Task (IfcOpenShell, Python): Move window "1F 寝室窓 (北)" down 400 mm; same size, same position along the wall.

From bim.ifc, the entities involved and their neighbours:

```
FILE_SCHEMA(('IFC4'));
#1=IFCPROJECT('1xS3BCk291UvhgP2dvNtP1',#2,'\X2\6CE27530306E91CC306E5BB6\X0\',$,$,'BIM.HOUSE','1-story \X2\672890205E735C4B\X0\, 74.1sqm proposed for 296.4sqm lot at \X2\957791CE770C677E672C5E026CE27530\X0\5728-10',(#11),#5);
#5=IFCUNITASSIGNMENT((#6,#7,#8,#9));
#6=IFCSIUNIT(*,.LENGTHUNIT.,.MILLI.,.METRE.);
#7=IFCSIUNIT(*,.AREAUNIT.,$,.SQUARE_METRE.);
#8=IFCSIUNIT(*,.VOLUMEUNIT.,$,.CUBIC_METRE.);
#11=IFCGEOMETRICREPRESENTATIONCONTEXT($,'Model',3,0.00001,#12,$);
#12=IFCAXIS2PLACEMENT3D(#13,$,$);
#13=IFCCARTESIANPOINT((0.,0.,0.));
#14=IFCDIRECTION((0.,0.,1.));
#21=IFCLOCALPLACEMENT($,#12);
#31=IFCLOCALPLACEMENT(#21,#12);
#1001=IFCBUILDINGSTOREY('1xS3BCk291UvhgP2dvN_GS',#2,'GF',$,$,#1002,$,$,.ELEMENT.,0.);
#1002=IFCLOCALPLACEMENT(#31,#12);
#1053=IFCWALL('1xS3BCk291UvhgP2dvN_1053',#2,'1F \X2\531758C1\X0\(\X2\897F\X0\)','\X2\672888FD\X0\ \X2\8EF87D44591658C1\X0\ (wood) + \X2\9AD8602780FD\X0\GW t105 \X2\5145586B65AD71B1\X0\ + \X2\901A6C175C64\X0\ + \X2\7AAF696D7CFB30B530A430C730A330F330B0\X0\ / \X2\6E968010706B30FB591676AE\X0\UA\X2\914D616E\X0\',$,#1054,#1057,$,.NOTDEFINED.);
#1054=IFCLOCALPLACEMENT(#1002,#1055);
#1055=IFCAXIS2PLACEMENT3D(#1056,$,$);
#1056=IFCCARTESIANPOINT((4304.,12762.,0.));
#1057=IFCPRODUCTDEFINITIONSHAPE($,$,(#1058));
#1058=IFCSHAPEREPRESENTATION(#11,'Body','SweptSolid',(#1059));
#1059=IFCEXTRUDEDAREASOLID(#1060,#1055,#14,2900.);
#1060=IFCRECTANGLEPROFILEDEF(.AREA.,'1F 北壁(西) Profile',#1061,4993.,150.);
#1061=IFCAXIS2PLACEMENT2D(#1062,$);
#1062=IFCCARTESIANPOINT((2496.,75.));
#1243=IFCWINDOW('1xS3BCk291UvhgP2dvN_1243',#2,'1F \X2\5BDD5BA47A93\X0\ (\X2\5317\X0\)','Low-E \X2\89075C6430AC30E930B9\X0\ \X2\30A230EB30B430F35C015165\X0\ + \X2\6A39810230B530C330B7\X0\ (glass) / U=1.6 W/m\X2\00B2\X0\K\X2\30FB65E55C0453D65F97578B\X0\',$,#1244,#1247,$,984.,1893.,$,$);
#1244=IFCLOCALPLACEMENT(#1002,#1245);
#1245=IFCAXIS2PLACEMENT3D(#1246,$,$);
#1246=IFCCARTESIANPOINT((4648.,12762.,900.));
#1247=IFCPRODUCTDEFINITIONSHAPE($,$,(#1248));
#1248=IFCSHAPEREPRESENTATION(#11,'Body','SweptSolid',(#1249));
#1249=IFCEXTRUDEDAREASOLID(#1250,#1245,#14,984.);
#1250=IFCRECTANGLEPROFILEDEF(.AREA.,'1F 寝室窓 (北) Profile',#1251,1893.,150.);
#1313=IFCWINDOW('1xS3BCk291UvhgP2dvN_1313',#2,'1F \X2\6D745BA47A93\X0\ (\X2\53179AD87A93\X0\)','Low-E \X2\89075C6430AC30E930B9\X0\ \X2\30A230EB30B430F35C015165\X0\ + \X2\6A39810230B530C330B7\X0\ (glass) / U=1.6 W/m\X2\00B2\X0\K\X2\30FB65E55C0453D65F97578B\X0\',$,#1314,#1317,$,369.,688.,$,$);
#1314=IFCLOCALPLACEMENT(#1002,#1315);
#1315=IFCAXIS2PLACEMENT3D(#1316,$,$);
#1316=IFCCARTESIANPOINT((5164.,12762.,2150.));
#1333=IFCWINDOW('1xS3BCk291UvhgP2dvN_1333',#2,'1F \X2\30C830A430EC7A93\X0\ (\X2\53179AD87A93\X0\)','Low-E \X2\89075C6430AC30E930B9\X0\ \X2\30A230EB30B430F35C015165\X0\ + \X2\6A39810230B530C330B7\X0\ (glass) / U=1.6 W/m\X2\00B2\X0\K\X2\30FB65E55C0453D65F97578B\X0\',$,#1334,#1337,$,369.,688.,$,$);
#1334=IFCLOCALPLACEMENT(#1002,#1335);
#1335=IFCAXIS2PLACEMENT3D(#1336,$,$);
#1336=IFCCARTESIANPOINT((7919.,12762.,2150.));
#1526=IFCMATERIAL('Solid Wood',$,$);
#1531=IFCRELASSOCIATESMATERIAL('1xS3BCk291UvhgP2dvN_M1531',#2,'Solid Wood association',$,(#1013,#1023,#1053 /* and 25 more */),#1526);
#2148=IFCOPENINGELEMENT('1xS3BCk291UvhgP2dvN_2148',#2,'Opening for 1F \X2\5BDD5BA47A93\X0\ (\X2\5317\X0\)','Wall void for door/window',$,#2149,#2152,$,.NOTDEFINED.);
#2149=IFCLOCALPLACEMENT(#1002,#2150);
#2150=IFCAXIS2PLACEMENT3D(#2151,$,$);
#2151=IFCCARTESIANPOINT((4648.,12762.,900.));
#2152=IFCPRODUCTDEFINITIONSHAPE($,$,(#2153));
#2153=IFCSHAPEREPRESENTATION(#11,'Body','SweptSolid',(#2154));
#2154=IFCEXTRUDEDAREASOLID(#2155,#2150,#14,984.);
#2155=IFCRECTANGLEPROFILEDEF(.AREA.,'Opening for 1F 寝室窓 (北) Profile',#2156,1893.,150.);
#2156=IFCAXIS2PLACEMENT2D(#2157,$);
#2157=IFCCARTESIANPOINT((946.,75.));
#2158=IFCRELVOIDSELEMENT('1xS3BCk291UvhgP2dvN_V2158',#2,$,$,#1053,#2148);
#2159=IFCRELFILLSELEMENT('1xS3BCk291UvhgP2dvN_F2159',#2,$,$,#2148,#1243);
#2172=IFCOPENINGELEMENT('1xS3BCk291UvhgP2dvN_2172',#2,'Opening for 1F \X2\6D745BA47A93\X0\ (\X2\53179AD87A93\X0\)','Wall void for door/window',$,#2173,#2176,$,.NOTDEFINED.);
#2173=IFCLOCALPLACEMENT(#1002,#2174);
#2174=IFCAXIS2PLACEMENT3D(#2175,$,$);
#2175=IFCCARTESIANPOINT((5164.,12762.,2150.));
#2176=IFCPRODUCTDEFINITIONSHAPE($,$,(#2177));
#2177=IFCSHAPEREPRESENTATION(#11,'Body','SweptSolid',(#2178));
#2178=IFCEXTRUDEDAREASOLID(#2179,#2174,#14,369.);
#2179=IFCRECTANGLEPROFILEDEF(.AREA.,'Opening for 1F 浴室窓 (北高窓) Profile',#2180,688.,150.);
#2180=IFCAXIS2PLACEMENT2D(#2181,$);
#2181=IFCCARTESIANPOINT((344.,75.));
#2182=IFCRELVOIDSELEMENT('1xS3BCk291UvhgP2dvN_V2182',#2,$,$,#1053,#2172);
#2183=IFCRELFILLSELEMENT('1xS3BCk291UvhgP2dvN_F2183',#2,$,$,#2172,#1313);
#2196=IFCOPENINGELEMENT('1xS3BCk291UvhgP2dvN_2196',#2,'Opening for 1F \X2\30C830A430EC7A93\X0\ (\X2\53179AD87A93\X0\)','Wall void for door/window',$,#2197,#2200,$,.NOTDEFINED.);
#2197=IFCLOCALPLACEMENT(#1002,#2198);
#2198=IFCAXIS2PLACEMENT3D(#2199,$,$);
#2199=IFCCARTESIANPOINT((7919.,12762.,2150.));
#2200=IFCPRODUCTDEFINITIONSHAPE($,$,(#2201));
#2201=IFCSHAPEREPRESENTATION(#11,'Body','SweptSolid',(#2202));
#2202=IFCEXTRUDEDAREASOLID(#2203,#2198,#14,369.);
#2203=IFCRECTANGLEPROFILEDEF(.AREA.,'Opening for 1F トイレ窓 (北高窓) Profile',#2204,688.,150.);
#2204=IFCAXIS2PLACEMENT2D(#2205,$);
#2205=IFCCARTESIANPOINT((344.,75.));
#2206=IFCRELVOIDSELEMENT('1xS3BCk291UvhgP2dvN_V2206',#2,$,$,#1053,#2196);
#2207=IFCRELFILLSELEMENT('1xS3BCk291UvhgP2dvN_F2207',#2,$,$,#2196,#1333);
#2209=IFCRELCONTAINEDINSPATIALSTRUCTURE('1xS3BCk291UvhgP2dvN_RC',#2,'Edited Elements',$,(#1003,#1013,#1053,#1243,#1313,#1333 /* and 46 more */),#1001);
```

```python
import numpy as np
import ifcopenshell
import ifcopenshell.api.geometry
import ifcopenshell.util.placement
import ifcopenshell.util.unit

model = ifcopenshell.open("bim.ifc")
unit_scale = ifcopenshell.util.unit.calculate_unit_scale(model)

window = model.by_id(1243)
opening = window.FillsVoids[0].RelatingOpeningElement
dz = -400.0

shift = np.array([0.0, 0.0, dz])
# The window is not placed relative to its opening, so move both.
for product in (opening, window):
    matrix = ifcopenshell.util.placement.get_local_placement(product.ObjectPlacement)
    matrix[:3, 3] += shift
    ifcopenshell.api.geometry.edit_object_placement(model, product=product, matrix=matrix, is_si=False)

print(f"moved by {dz * unit_scale:+.3f} m")

model.write("bim_updated.ifc")
```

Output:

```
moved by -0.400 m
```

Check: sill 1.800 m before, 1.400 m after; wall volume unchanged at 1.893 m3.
